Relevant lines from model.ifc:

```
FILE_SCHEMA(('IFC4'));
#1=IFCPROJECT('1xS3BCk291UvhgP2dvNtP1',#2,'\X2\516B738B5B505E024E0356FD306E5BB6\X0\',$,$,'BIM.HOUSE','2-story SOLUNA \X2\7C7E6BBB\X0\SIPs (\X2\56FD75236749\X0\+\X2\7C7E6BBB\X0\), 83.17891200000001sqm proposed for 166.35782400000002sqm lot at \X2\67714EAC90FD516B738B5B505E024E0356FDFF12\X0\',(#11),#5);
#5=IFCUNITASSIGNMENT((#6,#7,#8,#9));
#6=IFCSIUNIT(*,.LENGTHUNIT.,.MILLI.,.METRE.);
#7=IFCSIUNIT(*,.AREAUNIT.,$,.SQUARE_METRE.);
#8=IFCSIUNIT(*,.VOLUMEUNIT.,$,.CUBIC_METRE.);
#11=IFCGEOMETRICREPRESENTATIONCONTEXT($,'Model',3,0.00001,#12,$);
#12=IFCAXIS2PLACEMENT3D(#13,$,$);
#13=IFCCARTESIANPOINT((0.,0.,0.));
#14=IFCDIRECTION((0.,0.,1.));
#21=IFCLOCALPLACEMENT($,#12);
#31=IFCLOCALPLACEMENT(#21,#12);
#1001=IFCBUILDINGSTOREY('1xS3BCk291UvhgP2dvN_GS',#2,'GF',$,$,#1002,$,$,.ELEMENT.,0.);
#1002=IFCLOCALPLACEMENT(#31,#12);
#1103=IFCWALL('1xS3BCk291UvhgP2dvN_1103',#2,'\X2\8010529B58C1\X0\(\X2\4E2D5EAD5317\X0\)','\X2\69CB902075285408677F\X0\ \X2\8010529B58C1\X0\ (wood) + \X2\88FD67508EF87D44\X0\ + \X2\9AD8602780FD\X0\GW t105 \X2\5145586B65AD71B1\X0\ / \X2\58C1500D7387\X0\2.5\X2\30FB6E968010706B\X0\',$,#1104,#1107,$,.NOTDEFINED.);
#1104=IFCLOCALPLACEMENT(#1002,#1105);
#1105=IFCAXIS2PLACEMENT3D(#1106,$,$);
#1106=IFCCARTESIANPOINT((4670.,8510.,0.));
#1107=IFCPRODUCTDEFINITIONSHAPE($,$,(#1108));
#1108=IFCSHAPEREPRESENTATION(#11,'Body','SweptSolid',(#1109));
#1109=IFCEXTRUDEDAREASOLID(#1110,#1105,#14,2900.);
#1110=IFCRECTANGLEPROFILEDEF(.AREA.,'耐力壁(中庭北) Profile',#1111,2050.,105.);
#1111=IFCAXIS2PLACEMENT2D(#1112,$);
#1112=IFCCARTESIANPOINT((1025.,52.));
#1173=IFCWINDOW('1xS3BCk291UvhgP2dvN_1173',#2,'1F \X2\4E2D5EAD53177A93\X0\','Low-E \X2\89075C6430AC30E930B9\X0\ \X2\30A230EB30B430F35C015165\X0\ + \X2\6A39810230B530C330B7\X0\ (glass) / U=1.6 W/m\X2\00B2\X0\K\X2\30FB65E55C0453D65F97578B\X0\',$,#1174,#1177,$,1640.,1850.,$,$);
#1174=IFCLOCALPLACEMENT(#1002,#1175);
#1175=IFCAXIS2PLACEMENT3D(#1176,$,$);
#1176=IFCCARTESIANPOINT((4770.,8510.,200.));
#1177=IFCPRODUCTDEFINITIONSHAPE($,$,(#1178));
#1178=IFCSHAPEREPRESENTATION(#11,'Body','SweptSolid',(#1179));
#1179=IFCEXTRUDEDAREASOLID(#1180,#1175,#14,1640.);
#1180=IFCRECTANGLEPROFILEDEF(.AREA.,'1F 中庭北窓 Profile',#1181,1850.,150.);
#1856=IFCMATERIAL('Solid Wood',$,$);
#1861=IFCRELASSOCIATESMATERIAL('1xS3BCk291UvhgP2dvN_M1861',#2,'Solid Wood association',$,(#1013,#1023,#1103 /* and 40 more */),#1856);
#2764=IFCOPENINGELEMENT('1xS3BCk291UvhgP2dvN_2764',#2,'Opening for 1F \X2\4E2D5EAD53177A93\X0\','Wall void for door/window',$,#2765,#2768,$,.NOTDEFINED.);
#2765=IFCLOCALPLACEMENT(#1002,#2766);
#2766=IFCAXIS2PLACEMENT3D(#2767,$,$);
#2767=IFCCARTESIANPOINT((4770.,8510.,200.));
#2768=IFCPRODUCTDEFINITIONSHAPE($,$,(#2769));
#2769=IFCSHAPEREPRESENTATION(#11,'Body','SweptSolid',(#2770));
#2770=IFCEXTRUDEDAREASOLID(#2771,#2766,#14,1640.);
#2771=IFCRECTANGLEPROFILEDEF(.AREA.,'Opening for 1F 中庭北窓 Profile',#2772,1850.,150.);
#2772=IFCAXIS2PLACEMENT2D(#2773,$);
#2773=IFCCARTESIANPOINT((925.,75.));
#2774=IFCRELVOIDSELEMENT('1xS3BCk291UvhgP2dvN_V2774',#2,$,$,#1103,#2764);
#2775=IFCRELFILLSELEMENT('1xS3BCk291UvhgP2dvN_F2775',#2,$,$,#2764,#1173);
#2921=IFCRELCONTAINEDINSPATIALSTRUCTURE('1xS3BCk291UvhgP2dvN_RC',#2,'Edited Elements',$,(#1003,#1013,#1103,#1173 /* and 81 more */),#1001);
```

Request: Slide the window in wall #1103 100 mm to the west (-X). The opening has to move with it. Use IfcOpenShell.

```python
import ifcopenshell
import ifcopenshell.api.geometry
import ifcopenshell.util.placement
import ifcopenshell.util.unit

model = ifcopenshell.open("model.ifc")
unit_scale = ifcopenshell.util.unit.calculate_unit_scale(model)

window = model.by_guid("1xS3BCk291UvhgP2dvN_1173")
opening = window.FillsVoids[0].RelatingOpeningElement
wall = opening.VoidsElements[0].RelatingBuildingElement

wall_matrix = ifcopenshell.util.placement.get_local_placement(wall.ObjectPlacement)
shift = wall_matrix[:3, 0] * -0.1 / unit_scale
before = ifcopenshell.util.placement.get_local_placement(window.ObjectPlacement)[:3, 3].copy()

# The window is not placed relative to its opening, so move both.
for product in (opening, window):
    matrix = ifcopenshell.util.placement.get_local_placement(product.ObjectPlacement)
    matrix[:3, 3] += shift
    ifcopenshell.api.geometry.edit_object_placement(model, product=product, matrix=matrix, is_si=False)

after = ifcopenshell.util.placement.get_local_placement(window.ObjectPlacement)[:3, 3]
print("window moved by", (after - before).round(3) + 0.0)

model.write("model_edited.ifc")
```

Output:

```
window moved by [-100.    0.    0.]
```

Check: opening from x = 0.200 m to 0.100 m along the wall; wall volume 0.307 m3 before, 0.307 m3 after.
